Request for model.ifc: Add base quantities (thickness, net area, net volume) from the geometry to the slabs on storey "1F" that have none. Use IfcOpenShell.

First a look at what the model holds.

```python
import ifcopenshell
import ifcopenshell.util.element
import ifcopenshell.util.unit

model = ifcopenshell.open("model.ifc")
print(model.schema)
for unit_type in ("LENGTHUNIT", "AREAUNIT", "VOLUMEUNIT"):
    print(unit_type, ifcopenshell.util.unit.calculate_unit_scale(model, unit_type))
storey = next(s for s in model.by_type("IfcBuildingStorey") if s.Name == "1F")
slabs = [e for e in ifcopenshell.util.element.get_decomposition(storey) if e.is_a("IfcSlab")]
for e in sorted(slabs, key=lambda e: e.id()):
    print(e.id(), e.is_a(), e.Name, list(ifcopenshell.util.element.get_psets(e, qtos_only=True)), sep=" | ")
```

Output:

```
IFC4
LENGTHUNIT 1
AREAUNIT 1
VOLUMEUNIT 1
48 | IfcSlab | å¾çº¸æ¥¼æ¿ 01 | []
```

```python
import ifcopenshell
import ifcopenshell.api.pset
import ifcopenshell.geom
import ifcopenshell.util.element
import ifcopenshell.util.shape
import ifcopenshell.util.unit

model = ifcopenshell.open("model.ifc")
unit_scale = ifcopenshell.util.unit.calculate_unit_scale(model)
area_scale = ifcopenshell.util.unit.calculate_unit_scale(model, "AREAUNIT")
volume_scale = ifcopenshell.util.unit.calculate_unit_scale(model, "VOLUMEUNIT")
settings = ifcopenshell.geom.settings()

storey = next(s for s in model.by_type("IfcBuildingStorey") if s.Name == "1F")
slabs = [e for e in ifcopenshell.util.element.get_decomposition(storey) if e.is_a("IfcSlab")]

for e in sorted(slabs, key=lambda e: e.id()):
    if ifcopenshell.util.element.get_psets(e, qtos_only=True, should_inherit=False):
        continue
    # Geometry comes back in metres, in the element's own axes.
    shape = ifcopenshell.geom.create_shape(settings, e)
    values = {
        "Width": ifcopenshell.util.shape.get_z(shape.geometry) / unit_scale,
        "NetArea": ifcopenshell.util.shape.get_footprint_area(shape.geometry) / area_scale,
        "NetVolume": ifcopenshell.util.shape.get_volume(shape.geometry) / volume_scale,
    }
    qto = ifcopenshell.api.pset.add_qto(model, product=e, name="Qto_SlabBaseQuantities")
    ifcopenshell.api.pset.edit_qto(model, qto=qto, properties=values)
    print(e.id(), {k: round(v, 3) for k, v in values.items()})

model.write("model_v2.ifc")
```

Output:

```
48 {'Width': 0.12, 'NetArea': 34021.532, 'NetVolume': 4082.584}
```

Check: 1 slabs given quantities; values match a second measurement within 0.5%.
